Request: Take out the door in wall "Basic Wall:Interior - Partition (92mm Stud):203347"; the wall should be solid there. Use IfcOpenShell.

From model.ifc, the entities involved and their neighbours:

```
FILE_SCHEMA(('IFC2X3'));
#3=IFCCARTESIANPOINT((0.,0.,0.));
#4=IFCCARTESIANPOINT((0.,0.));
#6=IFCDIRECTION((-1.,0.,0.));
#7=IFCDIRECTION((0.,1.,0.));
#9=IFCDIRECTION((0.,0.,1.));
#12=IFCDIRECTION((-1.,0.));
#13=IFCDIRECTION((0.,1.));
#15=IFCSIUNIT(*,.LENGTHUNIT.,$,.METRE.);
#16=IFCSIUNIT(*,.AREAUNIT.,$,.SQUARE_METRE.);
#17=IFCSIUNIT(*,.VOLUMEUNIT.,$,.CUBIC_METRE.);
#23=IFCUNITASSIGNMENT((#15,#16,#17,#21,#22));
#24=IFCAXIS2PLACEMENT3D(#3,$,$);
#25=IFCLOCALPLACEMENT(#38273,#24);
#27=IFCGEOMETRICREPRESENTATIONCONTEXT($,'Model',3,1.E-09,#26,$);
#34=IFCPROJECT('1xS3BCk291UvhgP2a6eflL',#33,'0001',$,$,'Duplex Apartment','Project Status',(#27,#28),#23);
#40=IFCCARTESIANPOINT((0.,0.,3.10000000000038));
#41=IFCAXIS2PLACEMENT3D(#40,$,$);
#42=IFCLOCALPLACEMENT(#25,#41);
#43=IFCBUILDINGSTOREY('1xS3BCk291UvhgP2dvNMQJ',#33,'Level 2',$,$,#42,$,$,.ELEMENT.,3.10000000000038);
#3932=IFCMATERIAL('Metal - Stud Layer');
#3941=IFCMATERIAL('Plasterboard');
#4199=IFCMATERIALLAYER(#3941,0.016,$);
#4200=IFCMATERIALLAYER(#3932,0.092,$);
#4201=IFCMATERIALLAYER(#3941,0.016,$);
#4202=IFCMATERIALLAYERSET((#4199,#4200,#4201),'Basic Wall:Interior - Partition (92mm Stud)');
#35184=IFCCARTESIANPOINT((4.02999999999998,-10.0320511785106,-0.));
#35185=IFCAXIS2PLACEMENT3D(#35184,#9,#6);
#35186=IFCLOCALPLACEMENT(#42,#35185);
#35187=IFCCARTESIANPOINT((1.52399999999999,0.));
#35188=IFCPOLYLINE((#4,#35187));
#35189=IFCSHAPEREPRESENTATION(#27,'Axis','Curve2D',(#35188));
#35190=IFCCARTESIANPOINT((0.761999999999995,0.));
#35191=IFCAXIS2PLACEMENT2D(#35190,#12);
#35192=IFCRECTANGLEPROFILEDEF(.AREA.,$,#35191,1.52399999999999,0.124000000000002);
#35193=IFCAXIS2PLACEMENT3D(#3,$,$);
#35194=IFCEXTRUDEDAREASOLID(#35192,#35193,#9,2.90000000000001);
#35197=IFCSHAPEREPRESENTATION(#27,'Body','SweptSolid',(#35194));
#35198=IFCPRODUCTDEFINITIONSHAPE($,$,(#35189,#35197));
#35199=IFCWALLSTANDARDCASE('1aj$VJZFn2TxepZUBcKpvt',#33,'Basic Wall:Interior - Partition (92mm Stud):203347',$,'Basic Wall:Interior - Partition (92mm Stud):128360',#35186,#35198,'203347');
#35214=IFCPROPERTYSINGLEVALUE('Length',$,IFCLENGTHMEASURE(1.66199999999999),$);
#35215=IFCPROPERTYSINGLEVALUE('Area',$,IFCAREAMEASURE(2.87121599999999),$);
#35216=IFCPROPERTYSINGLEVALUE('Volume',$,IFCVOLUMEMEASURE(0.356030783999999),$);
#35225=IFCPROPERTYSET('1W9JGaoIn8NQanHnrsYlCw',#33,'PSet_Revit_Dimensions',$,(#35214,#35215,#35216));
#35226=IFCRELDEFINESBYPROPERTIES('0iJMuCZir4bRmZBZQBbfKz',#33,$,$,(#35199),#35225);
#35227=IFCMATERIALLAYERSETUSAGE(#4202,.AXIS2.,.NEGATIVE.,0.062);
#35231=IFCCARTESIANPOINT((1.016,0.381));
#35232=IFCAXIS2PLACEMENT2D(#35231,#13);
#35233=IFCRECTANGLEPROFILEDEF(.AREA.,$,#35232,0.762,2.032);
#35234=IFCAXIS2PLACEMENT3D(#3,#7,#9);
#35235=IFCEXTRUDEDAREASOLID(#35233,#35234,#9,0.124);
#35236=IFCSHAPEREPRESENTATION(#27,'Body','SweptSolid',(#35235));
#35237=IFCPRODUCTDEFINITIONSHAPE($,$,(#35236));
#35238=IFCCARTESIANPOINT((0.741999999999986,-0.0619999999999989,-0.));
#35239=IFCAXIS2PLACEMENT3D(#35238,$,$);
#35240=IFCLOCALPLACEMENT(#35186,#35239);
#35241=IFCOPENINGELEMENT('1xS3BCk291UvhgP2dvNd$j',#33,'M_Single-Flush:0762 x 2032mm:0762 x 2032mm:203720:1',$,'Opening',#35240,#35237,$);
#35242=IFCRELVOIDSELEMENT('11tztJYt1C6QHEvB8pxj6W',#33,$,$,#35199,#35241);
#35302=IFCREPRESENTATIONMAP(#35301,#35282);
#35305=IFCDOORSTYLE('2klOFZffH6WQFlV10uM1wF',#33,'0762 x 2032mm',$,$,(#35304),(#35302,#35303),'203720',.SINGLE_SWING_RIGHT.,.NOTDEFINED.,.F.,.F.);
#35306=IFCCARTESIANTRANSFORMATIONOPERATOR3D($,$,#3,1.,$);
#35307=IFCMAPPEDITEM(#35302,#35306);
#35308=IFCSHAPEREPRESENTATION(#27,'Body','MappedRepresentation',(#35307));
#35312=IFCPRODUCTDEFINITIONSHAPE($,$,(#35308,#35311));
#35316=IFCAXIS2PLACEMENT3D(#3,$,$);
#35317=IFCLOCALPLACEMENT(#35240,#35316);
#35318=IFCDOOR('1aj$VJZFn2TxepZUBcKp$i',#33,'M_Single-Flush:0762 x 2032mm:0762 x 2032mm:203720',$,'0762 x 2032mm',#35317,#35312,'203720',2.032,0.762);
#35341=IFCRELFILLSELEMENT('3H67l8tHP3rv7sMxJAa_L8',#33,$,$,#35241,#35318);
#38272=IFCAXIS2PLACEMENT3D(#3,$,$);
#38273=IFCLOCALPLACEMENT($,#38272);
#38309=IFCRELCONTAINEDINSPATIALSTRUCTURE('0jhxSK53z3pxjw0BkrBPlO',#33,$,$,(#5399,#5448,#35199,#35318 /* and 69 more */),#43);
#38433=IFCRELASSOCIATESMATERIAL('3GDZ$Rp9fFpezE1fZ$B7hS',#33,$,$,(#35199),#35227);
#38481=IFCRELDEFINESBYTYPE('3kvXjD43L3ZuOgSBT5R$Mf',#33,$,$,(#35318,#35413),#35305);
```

```python
import ifcopenshell
import ifcopenshell.api.feature
import ifcopenshell.api.pset
import ifcopenshell.api.root
import ifcopenshell.geom
import ifcopenshell.util.element
import ifcopenshell.util.shape
import ifcopenshell.util.unit

model = ifcopenshell.open("model.ifc")
area_scale = ifcopenshell.util.unit.calculate_unit_scale(model, "AREAUNIT")
volume_scale = ifcopenshell.util.unit.calculate_unit_scale(model, "VOLUMEUNIT")
settings = ifcopenshell.geom.settings()


def volume(element):
    """Net volume in cubic metres, openings subtracted."""
    shape = ifcopenshell.geom.create_shape(settings, element)
    return ifcopenshell.util.shape.get_volume(shape.geometry)


door = model.by_guid("1aj$VJZFn2TxepZUBcKp$i")
opening = door.FillsVoids[0].RelatingOpeningElement
wall = opening.VoidsElements[0].RelatingBuildingElement
before = volume(wall)

ifcopenshell.api.root.remove_product(model, product=door)
ifcopenshell.api.feature.remove_feature(model, feature=opening)

after = volume(wall)
thickness = 0.124  # wall thickness in metres

# Update the wall's stored quantities.
pset = model.by_id(ifcopenshell.util.element.get_pset(wall, "PSet_Revit_Dimensions", should_inherit=False)["id"])
ifcopenshell.api.pset.edit_pset(model, pset=pset, properties={
    "Area": model.create_entity("IfcAreaMeasure", after / thickness / area_scale),
    "Volume": model.create_entity("IfcVolumeMeasure", after / volume_scale),
})

print(f"wall volume {before:.3f} -> {after:.3f} m3")

model.write("model-out.ifc")
```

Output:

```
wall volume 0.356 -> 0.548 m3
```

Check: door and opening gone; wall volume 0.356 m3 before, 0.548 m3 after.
